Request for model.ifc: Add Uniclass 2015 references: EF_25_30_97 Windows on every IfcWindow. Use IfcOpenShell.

First a look at what the model holds.

```python
import ifcopenshell

model = ifcopenshell.open("model.ifc")
print(model.schema)
print("classifications:", [c.Name for c in model.by_type("IfcClassification")])
for ifc_class in ("IfcDoor", "IfcRoof", "IfcStair", "IfcWall", "IfcWindow"):
    print(ifc_class, len(model.by_type(ifc_class)))
```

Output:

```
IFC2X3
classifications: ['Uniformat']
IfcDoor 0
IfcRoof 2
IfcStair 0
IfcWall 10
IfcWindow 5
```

```python
import ifcopenshell
import ifcopenshell.api.classification

model = ifcopenshell.open("model.ifc")

# IFC2X3 requires Source and Edition and has no link from the project to the system.
system = model.create_entity("IfcClassification", Source="NBS", Edition="2015", Name="Uniclass 2015")

codes = {
    "IfcWindow": ("EF_25_30_97", "Windows"),
}
for ifc_class, (code, name) in codes.items():
    products = model.by_type(ifc_class)
    ifcopenshell.api.classification.add_reference(
        model, products=products, classification=system, identification=code, name=name
    )
    print(code, len(products))

model.write("model_updated.ifc")
```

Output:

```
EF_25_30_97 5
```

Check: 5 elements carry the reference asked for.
